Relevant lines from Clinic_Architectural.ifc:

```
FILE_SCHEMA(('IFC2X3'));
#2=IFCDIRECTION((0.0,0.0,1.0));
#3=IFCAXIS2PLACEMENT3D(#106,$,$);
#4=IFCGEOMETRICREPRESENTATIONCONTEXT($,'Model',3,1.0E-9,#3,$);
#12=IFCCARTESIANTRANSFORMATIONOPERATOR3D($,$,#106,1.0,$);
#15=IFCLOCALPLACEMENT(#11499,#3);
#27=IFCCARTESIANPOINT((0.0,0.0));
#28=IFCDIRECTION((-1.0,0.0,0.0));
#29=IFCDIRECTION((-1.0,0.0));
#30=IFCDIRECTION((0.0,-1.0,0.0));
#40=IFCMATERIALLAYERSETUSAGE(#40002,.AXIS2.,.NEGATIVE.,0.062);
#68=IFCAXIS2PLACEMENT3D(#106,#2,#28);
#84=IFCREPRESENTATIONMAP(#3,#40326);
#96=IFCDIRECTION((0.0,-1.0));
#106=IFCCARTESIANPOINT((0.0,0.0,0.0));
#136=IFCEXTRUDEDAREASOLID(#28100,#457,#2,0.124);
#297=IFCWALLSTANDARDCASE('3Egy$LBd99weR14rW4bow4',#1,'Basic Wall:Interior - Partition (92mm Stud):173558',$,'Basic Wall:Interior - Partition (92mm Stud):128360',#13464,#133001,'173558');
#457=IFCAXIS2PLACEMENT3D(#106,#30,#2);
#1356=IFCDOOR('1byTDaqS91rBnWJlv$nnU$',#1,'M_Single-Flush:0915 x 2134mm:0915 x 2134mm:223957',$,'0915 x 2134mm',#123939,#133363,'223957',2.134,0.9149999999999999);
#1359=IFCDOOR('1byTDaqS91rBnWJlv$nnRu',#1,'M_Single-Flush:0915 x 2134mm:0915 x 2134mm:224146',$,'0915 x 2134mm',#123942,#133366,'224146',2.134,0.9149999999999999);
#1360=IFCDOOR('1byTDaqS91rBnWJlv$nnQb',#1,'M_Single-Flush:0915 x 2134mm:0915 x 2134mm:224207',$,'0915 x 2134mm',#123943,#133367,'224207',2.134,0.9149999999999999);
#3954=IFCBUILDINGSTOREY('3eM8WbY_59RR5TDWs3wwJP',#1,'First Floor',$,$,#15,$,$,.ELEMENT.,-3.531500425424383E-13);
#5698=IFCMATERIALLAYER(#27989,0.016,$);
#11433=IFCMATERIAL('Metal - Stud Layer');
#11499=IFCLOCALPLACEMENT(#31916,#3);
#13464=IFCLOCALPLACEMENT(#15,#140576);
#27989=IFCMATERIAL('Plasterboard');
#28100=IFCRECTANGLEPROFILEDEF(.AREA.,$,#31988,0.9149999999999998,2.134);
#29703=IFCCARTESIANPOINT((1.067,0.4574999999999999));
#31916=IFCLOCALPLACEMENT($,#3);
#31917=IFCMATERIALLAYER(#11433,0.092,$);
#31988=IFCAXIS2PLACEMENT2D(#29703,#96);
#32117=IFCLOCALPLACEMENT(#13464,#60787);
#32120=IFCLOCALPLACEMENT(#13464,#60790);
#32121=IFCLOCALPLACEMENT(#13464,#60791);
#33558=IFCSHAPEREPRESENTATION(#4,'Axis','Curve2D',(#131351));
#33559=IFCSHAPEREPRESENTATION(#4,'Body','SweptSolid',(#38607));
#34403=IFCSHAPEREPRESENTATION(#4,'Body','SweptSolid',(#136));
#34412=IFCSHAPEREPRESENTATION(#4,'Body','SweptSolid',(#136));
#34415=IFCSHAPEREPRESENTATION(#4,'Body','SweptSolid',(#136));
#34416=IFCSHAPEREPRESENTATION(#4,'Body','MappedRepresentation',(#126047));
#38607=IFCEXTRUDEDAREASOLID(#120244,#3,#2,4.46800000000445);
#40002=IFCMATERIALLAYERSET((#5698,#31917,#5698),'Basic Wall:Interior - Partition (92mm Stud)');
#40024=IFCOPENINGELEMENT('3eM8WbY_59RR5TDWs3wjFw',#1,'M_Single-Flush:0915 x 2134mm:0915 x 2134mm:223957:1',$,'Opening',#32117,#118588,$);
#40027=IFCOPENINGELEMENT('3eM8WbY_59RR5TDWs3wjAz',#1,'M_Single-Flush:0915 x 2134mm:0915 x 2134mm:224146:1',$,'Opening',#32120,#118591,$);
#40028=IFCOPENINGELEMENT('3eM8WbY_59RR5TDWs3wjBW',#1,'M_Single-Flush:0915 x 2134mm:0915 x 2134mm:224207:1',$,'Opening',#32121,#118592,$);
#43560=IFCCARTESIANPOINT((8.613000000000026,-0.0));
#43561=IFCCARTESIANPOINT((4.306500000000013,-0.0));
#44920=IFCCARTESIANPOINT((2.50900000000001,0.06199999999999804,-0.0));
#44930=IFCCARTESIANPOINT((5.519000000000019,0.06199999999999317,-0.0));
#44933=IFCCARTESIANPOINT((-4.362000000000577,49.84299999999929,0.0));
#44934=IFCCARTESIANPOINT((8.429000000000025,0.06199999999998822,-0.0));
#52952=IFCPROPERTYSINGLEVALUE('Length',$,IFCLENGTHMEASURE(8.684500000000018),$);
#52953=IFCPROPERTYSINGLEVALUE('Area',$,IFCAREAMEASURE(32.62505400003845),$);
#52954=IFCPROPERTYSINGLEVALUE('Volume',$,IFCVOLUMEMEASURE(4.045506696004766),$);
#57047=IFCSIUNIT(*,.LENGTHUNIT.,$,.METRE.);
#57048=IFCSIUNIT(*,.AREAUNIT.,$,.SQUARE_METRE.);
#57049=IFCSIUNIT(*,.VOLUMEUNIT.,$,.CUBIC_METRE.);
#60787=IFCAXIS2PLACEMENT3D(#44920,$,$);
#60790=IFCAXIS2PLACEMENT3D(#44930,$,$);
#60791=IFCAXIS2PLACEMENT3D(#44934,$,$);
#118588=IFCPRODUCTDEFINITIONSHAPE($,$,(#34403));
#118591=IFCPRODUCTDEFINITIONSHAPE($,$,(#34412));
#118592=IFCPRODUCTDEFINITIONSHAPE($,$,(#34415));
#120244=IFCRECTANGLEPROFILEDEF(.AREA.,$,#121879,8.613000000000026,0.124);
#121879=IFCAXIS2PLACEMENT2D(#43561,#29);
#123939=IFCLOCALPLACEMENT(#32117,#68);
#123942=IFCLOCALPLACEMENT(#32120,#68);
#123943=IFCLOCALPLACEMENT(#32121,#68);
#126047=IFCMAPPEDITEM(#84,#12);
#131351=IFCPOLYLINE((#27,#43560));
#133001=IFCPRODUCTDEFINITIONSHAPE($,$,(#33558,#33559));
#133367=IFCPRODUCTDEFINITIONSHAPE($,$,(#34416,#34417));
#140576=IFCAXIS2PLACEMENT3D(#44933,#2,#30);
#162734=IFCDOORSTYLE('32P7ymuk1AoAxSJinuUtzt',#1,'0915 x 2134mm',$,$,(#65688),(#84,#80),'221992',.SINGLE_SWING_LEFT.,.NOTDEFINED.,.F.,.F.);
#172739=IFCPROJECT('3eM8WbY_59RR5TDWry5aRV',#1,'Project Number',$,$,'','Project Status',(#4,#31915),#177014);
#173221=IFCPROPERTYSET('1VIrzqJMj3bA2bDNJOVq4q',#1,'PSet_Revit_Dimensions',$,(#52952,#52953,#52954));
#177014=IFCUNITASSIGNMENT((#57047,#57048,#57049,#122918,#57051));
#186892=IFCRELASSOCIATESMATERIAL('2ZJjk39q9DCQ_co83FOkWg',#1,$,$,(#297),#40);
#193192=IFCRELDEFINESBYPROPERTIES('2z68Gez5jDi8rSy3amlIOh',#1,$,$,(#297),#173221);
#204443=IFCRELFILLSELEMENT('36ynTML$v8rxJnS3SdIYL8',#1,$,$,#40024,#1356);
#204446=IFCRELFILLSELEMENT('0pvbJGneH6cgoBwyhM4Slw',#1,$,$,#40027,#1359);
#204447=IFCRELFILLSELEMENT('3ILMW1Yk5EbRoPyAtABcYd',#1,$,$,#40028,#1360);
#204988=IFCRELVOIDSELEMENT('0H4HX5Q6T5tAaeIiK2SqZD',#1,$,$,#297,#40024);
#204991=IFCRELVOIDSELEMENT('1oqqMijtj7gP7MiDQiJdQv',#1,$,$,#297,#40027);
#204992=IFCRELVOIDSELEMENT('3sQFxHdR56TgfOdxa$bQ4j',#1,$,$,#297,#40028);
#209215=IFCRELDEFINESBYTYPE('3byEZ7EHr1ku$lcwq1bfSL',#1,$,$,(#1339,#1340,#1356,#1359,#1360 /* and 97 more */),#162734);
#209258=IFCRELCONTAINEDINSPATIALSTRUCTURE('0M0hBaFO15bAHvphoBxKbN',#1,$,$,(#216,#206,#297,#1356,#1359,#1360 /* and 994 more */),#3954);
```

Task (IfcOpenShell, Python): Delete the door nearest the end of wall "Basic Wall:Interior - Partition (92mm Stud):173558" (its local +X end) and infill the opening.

```python
import ifcopenshell
import ifcopenshell.api.feature
import ifcopenshell.api.pset
import ifcopenshell.api.root
import ifcopenshell.geom
import ifcopenshell.util.element
import ifcopenshell.util.shape
import ifcopenshell.util.unit

model = ifcopenshell.open("Clinic_Architectural.ifc")
area_scale = ifcopenshell.util.unit.calculate_unit_scale(model, "AREAUNIT")
volume_scale = ifcopenshell.util.unit.calculate_unit_scale(model, "VOLUMEUNIT")
settings = ifcopenshell.geom.settings()


def volume(element):
    """Net volume in cubic metres, openings subtracted."""
    shape = ifcopenshell.geom.create_shape(settings, element)
    return ifcopenshell.util.shape.get_volume(shape.geometry)


door = model.by_guid("1byTDaqS91rBnWJlv$nnQb")
opening = door.FillsVoids[0].RelatingOpeningElement
wall = opening.VoidsElements[0].RelatingBuildingElement
before = volume(wall)

ifcopenshell.api.root.remove_product(model, product=door)
ifcopenshell.api.feature.remove_feature(model, feature=opening)

after = volume(wall)
thickness = 0.124  # wall thickness in metres

# Update the wall's stored quantities.
pset = model.by_id(ifcopenshell.util.element.get_pset(wall, "PSet_Revit_Dimensions", should_inherit=False)["id"])
ifcopenshell.api.pset.edit_pset(model, pset=pset, properties={
    "Area": model.create_entity("IfcAreaMeasure", after / thickness / area_scale),
    "Volume": model.create_entity("IfcVolumeMeasure", after / volume_scale),
})

print(f"wall volume {before:.3f} -> {after:.3f} m3")

model.write("Clinic_Architectural_edited.ifc")
```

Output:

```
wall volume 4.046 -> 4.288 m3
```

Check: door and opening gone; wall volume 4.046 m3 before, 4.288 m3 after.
